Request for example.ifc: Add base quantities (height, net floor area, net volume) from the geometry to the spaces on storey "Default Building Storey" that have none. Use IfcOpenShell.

First a look at what the model holds.

```python
import ifcopenshell
import ifcopenshell.util.element
import ifcopenshell.util.unit

model = ifcopenshell.open("example.ifc")
print(model.schema)
for unit_type in ("LENGTHUNIT", "AREAUNIT", "VOLUMEUNIT"):
    print(unit_type, ifcopenshell.util.unit.calculate_unit_scale(model, unit_type))
storey = next(s for s in model.by_type("IfcBuildingStorey") if s.Name == "Default Building Storey")
spaces = [e for e in ifcopenshell.util.element.get_decomposition(storey) if e.is_a("IfcSpace")]
for e in sorted(spaces, key=lambda e: e.id()):
    print(e.id(), e.is_a(), e.Name, list(ifcopenshell.util.element.get_psets(e, qtos_only=True)), sep=" | ")
```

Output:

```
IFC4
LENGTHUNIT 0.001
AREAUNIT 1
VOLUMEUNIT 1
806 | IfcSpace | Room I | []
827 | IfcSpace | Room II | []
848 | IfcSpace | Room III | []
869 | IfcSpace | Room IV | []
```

```python
import ifcopenshell
import ifcopenshell.api.pset
import ifcopenshell.geom
import ifcopenshell.util.element
import ifcopenshell.util.shape
import ifcopenshell.util.unit

model = ifcopenshell.open("example.ifc")
unit_scale = ifcopenshell.util.unit.calculate_unit_scale(model)
area_scale = ifcopenshell.util.unit.calculate_unit_scale(model, "AREAUNIT")
volume_scale = ifcopenshell.util.unit.calculate_unit_scale(model, "VOLUMEUNIT")
settings = ifcopenshell.geom.settings()

storey = next(s for s in model.by_type("IfcBuildingStorey") if s.Name == "Default Building Storey")
spaces = [e for e in ifcopenshell.util.element.get_decomposition(storey) if e.is_a("IfcSpace")]

for e in sorted(spaces, key=lambda e: e.id()):
    if ifcopenshell.util.element.get_psets(e, qtos_only=True, should_inherit=False):
        continue
    # Geometry comes back in metres, in the element's own axes.
    shape = ifcopenshell.geom.create_shape(settings, e)
    values = {
        "Height": ifcopenshell.util.shape.get_z(shape.geometry) / unit_scale,
        "NetFloorArea": ifcopenshell.util.shape.get_footprint_area(shape.geometry) / area_scale,
        "NetVolume": ifcopenshell.util.shape.get_volume(shape.geometry) / volume_scale,
    }
    qto = ifcopenshell.api.pset.add_qto(model, product=e, name="Qto_SpaceBaseQuantities")
    ifcopenshell.api.pset.edit_qto(model, qto=qto, properties=values)
    print(e.id(), {k: round(v, 3) for k, v in values.items()})

model.write("example_v2.ifc")
```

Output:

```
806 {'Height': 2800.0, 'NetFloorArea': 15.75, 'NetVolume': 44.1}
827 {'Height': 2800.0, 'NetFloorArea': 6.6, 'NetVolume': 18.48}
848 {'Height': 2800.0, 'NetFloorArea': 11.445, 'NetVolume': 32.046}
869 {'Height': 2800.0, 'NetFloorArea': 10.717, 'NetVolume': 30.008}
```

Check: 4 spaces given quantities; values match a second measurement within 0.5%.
